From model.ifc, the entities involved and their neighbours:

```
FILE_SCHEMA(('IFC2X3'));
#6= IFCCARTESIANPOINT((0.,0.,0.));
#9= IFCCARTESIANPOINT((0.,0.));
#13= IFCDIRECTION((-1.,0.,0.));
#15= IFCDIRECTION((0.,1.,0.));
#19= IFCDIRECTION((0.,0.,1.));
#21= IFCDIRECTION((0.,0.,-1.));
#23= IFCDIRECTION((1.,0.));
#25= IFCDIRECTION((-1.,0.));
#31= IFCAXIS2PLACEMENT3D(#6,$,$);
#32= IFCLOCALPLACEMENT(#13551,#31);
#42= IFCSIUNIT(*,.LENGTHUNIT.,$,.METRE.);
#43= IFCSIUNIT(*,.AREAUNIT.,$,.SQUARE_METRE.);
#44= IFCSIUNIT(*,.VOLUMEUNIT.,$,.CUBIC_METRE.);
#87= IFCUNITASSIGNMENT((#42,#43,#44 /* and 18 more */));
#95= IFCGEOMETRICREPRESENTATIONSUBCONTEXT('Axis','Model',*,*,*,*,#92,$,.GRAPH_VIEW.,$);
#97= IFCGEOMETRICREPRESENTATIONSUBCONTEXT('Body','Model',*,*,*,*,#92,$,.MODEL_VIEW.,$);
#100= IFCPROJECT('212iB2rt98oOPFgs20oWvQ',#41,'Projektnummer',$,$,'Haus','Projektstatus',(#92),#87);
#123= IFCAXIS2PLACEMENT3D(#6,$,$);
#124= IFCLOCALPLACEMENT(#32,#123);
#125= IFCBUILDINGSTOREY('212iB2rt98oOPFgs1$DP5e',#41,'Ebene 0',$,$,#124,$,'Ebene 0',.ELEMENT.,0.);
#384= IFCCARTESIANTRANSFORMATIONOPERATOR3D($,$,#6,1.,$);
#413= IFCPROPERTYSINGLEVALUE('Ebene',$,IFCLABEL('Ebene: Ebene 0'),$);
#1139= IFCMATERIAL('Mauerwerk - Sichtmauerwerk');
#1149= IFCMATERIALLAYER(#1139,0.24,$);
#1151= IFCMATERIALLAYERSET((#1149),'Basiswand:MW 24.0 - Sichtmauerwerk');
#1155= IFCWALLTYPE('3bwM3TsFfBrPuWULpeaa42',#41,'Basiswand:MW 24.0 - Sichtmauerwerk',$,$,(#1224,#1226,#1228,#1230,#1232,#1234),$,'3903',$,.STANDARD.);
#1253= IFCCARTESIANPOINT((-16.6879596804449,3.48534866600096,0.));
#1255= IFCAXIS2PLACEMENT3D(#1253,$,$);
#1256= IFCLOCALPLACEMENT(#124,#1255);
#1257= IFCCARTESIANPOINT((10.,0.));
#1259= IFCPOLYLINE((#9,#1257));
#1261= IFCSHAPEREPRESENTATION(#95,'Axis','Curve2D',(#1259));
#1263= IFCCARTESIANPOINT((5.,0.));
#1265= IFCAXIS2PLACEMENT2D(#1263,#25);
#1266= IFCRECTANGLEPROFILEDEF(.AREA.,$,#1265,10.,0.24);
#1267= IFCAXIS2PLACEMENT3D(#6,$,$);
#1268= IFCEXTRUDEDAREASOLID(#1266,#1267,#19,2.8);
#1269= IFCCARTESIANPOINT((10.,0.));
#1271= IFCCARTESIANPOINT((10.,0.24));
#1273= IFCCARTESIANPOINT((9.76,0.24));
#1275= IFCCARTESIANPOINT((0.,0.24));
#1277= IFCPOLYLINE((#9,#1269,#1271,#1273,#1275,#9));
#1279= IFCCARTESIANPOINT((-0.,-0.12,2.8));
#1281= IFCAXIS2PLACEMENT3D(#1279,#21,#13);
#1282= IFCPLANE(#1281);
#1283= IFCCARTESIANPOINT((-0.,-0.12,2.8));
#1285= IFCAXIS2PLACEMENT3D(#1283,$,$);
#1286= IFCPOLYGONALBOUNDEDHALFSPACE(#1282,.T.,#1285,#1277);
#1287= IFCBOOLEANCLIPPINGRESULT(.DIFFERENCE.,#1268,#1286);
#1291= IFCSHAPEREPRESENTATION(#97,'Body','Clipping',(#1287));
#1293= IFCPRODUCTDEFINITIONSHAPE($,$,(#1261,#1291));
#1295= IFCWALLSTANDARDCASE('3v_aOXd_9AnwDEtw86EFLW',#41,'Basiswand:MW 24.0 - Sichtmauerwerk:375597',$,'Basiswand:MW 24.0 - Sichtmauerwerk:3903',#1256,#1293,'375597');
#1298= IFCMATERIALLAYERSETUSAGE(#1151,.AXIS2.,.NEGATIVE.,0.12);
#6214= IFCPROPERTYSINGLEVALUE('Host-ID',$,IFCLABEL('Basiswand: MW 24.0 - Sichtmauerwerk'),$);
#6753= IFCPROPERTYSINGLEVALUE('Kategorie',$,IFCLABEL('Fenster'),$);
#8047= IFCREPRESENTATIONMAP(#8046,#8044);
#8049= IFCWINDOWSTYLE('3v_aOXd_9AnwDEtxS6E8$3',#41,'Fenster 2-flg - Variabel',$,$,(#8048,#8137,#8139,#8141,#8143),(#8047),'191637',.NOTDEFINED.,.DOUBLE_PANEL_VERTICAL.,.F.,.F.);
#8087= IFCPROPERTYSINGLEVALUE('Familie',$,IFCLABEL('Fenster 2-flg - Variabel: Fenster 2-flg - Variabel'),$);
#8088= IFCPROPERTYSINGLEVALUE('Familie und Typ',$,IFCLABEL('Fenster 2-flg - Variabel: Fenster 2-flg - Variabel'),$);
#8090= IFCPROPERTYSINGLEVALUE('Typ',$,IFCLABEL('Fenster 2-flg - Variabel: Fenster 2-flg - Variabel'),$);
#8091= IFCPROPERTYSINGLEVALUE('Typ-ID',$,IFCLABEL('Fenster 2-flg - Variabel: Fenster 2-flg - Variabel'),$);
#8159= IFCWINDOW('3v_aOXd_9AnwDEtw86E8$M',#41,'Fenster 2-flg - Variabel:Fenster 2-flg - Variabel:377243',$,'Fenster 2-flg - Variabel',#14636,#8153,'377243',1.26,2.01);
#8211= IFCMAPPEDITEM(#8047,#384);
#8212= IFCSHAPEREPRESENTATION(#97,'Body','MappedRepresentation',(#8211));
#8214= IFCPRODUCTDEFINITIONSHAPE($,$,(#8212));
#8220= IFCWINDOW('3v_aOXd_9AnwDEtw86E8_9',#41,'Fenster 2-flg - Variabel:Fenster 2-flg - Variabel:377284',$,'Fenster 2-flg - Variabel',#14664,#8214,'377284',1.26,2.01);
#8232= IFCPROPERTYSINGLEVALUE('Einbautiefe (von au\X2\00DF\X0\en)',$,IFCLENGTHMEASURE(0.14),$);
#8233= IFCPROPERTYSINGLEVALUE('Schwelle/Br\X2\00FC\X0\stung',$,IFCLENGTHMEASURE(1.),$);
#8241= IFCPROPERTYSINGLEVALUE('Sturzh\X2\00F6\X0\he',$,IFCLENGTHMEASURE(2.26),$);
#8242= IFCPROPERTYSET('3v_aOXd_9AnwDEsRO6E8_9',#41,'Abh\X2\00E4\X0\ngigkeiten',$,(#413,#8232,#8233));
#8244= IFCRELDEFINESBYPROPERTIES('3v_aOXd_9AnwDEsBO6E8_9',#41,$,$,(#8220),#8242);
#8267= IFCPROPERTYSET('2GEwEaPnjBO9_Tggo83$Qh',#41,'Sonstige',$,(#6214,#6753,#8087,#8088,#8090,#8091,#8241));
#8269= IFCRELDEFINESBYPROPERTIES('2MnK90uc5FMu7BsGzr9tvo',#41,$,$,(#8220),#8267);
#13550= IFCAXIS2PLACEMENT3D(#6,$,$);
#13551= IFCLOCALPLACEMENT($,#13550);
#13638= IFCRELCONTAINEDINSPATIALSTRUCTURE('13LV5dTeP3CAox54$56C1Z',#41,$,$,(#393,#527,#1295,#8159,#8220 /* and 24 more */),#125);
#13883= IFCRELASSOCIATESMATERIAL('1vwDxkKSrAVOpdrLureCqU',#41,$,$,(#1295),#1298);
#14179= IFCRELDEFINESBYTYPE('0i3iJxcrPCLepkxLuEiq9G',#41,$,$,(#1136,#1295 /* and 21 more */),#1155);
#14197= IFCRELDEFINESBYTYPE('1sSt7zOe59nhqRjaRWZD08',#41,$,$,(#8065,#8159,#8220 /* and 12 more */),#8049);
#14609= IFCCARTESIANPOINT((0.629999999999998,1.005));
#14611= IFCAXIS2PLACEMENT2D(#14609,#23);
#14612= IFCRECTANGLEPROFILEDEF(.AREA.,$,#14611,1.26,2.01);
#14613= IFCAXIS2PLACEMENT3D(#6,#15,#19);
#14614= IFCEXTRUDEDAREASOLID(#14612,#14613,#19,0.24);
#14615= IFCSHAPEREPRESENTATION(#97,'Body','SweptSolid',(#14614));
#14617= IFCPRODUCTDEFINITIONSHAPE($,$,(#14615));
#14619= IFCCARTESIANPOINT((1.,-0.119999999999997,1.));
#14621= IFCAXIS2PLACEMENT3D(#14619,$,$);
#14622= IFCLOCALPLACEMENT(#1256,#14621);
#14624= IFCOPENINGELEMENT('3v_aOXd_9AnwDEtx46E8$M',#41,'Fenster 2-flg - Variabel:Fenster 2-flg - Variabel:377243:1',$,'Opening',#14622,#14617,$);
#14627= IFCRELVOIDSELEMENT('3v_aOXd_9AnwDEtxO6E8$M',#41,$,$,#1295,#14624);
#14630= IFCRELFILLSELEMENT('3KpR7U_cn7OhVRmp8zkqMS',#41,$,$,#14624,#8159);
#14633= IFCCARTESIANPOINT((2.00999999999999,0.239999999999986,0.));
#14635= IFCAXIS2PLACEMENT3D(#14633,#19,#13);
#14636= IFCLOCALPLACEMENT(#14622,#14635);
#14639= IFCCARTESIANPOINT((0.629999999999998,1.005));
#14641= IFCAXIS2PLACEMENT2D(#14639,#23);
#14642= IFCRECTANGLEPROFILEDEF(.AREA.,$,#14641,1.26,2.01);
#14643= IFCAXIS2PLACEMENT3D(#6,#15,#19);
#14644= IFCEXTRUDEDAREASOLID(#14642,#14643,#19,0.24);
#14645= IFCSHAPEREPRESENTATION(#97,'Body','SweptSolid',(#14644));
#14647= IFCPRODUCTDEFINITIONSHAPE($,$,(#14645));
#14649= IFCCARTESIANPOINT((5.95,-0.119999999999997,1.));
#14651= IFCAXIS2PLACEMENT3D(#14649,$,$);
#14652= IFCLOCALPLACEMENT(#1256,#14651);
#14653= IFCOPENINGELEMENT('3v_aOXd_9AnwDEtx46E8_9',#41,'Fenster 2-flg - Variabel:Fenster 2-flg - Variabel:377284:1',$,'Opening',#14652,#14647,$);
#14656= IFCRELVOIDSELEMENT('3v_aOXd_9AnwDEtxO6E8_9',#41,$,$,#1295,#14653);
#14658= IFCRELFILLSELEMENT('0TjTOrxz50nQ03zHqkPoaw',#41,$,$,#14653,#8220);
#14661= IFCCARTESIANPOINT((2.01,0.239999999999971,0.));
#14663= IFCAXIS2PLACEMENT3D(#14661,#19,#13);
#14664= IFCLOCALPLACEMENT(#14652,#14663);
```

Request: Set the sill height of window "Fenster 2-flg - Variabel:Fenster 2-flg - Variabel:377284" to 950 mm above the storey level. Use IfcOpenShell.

```python
import numpy as np
import ifcopenshell
import ifcopenshell.api.geometry
import ifcopenshell.api.pset
import ifcopenshell.geom
import ifcopenshell.util.element
import ifcopenshell.util.placement
import ifcopenshell.util.shape
import ifcopenshell.util.unit

model = ifcopenshell.open("model.ifc")
unit_scale = ifcopenshell.util.unit.calculate_unit_scale(model)

window = model.by_guid("3v_aOXd_9AnwDEtw86E8_9")
opening = window.FillsVoids[0].RelatingOpeningElement
storey = ifcopenshell.util.element.get_container(window, ifc_class="IfcBuildingStorey")
level = ifcopenshell.util.placement.get_local_placement(storey.ObjectPlacement)[2, 3]

# The opening's origin need not be at the sill, so measure its lowest point.
shape = ifcopenshell.geom.create_shape(ifcopenshell.geom.settings(), opening)
bottom = ifcopenshell.util.shape.get_shape_bottom_elevation(shape, shape.geometry) / unit_scale
dz = level + 0.95 / unit_scale - bottom

shift = np.array([0.0, 0.0, dz])
# The window is placed relative to its opening, so it follows when the opening moves.
matrix = ifcopenshell.util.placement.get_local_placement(opening.ObjectPlacement)
matrix[:3, 3] += shift
ifcopenshell.api.geometry.edit_object_placement(
    model, product=opening, matrix=matrix, is_si=False, should_transform_children=True
)

# Keep the stored heights in step.
pset = model.by_id(ifcopenshell.util.element.get_pset(window, "Abhängigkeiten", should_inherit=False)["id"])
ifcopenshell.api.pset.edit_pset(model, pset=pset, properties={
    "Schwelle/Brüstung": model.create_entity("IfcLengthMeasure", ifcopenshell.util.element.get_pset(window, "Abhängigkeiten", "Schwelle/Brüstung") + dz),
})
pset = model.by_id(ifcopenshell.util.element.get_pset(window, "Sonstige", should_inherit=False)["id"])
ifcopenshell.api.pset.edit_pset(model, pset=pset, properties={
    "Sturzhöhe": model.create_entity("IfcLengthMeasure", ifcopenshell.util.element.get_pset(window, "Sonstige", "Sturzhöhe") + dz),
})

print(f"moved by {dz * unit_scale:+.3f} m")

model.write("model_rev.ifc")
```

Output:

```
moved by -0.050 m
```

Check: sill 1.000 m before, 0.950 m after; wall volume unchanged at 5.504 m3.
